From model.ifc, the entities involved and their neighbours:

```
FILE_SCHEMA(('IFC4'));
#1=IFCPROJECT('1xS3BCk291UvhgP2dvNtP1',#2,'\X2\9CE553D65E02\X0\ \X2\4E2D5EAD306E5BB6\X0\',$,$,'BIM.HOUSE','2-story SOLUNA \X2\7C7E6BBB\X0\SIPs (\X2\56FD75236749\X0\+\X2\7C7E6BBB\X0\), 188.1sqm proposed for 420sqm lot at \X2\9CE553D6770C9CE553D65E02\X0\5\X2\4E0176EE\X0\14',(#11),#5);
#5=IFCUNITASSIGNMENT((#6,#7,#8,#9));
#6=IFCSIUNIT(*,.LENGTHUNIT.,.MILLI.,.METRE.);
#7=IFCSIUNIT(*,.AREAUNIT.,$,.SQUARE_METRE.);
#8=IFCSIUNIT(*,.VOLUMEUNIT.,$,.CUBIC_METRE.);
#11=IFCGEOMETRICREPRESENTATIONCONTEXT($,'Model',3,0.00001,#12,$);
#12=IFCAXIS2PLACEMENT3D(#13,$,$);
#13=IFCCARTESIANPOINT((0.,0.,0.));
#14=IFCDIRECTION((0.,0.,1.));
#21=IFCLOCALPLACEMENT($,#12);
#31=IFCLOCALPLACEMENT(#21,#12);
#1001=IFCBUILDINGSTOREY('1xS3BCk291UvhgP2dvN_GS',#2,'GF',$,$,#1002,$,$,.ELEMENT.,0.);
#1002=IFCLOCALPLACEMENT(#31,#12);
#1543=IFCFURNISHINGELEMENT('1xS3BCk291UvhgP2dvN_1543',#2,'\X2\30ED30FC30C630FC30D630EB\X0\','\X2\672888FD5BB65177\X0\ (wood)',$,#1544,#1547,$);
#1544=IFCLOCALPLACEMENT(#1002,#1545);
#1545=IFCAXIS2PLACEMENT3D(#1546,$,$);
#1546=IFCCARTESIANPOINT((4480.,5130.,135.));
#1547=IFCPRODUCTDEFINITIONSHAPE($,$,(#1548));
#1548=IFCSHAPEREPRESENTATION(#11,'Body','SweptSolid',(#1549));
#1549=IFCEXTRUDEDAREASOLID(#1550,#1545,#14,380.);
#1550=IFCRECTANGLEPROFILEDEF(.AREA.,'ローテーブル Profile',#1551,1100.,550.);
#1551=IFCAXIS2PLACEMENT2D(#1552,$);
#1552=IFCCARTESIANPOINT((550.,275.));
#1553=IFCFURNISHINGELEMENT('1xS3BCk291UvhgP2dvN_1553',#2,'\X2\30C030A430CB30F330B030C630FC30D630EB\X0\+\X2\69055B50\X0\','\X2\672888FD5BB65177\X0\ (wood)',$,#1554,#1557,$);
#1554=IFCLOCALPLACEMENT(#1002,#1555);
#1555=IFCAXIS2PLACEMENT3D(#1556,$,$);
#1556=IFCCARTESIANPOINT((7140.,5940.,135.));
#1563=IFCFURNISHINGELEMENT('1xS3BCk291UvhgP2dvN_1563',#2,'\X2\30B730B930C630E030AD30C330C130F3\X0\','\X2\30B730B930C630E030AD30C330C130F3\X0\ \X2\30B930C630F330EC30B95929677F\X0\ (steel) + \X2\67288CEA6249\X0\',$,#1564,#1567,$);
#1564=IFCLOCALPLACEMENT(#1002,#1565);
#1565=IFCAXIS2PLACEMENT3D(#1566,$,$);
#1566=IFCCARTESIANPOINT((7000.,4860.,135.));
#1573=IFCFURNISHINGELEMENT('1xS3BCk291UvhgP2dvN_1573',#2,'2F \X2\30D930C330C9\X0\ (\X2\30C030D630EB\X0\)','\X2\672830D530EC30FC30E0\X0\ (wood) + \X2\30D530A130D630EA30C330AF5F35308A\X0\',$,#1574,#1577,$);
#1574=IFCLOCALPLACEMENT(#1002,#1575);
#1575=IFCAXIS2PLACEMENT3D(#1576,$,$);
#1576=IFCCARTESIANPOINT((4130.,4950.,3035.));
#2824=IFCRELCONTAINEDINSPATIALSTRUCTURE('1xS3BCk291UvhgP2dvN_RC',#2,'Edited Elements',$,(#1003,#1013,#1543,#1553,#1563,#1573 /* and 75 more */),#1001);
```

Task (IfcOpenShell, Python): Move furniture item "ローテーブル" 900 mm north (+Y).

```python
import ifcopenshell
import ifcopenshell.api.geometry
import ifcopenshell.util.placement
import ifcopenshell.util.unit

model = ifcopenshell.open("model.ifc")
unit_scale = ifcopenshell.util.unit.calculate_unit_scale(model)

item = model.by_guid("1xS3BCk291UvhgP2dvN_1543")
matrix = ifcopenshell.util.placement.get_local_placement(item.ObjectPlacement)
matrix[1, 3] += 0.9 / unit_scale
ifcopenshell.api.geometry.edit_object_placement(model, product=item, matrix=matrix, is_si=False)

print(ifcopenshell.util.placement.get_local_placement(item.ObjectPlacement).round(3) + 0.0)

model.write("model-out.ifc")
```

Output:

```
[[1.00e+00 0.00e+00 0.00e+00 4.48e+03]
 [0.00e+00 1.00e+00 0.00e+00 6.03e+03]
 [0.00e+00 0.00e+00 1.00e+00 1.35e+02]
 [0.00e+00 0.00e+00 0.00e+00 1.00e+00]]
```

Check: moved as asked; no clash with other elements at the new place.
